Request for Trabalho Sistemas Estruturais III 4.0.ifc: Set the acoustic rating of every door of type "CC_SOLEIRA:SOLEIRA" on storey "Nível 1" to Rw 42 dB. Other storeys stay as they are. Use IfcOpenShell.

First a look at what the model holds.

```python
import ifcopenshell
import ifcopenshell.util.element

model = ifcopenshell.open("Trabalho Sistemas Estruturais III 4.0.ifc")
print(model.schema)
storey = next(s for s in model.by_type("IfcBuildingStorey") if s.Name == "Nível 1")
doors = [e for e in ifcopenshell.util.element.get_decomposition(storey) if e.is_a("IfcDoor")]
seen = {}
for e in doors:
    element_type = ifcopenshell.util.element.get_type(e)
    key = (element_type.Name if element_type != e and element_type else None, ifcopenshell.util.element.get_pset(e, "Pset_DoorCommon", "AcousticRating"))
    seen[key] = seen.get(key, 0) + 1
for (name, value), count in sorted(seen.items(), key=str):
    print(count, "x", name, "|", value)
```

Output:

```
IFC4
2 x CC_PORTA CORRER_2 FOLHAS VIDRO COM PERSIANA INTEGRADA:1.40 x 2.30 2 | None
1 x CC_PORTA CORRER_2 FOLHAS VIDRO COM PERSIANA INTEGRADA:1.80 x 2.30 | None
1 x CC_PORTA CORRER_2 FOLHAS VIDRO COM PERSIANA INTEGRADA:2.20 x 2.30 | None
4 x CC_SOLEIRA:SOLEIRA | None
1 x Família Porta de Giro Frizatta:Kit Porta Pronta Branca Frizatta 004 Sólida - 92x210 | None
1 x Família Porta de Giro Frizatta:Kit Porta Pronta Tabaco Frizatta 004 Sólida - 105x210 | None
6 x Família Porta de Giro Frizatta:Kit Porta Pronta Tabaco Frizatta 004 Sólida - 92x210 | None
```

```python
import ifcopenshell
import ifcopenshell.api.pset
import ifcopenshell.util.element

model = ifcopenshell.open("Trabalho Sistemas Estruturais III 4.0.ifc")

storey = next(s for s in model.by_type("IfcBuildingStorey") if s.Name == "Nível 1")
doors = [e for e in ifcopenshell.util.element.get_decomposition(storey) if e.is_a("IfcDoor")]

count = 0
for e in doors:
    element_type = ifcopenshell.util.element.get_type(e)
    if element_type in (None, e) or element_type.Name != "CC_SOLEIRA:SOLEIRA":
        continue
    # add_pset returns the element's existing set when there is one.
    pset = ifcopenshell.api.pset.add_pset(model, product=e, name="Pset_DoorCommon")
    ifcopenshell.api.pset.edit_pset(model, pset=pset, properties={"AcousticRating": "Rw 42 dB"})
    count += 1

print(count, "doors updated")

model.write("Trabalho Sistemas Estruturais III 4.0_edited.ifc")
```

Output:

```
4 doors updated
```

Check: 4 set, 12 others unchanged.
